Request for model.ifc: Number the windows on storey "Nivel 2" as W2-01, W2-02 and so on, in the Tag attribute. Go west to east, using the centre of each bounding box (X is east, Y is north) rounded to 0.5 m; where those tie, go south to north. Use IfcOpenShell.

First a look at what the model holds.

```python
import ifcopenshell
import ifcopenshell.util.element
import ifcopenshell.util.placement

model = ifcopenshell.open("model.ifc")
print(model.schema)
storey = next(s for s in model.by_type("IfcBuildingStorey") if s.Name == "Nivel 2")
windows = [e for e in ifcopenshell.util.element.get_decomposition(storey) if e.is_a("IfcWindow")]
for e in sorted(windows, key=lambda e: e.id()):
    origin = ifcopenshell.util.placement.get_local_placement(e.ObjectPlacement)[:3, 3]
    print(e.id(), e.Tag, e.Name, origin.round(2) + 0.0, sep=" | ")
```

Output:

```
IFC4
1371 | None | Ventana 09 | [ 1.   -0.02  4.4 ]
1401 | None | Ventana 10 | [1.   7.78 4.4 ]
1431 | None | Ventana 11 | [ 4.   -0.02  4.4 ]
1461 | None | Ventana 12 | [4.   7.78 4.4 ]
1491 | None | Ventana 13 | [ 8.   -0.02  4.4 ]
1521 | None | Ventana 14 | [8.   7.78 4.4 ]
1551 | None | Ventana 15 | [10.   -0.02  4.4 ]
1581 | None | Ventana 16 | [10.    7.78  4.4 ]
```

```python
import ifcopenshell
import ifcopenshell.geom
import ifcopenshell.util.element
import ifcopenshell.util.shape

model = ifcopenshell.open("model.ifc")
settings = ifcopenshell.geom.settings()
settings.set("use-world-coords", True)


def centre(element):
    shape = ifcopenshell.geom.create_shape(settings, element)
    return ifcopenshell.util.shape.get_bbox_centroid(shape.geometry)


storey = next(s for s in model.by_type("IfcBuildingStorey") if s.Name == "Nivel 2")
windows = [e for e in ifcopenshell.util.element.get_decomposition(storey) if e.is_a("IfcWindow")]

# Insertion points can sit at a corner or the storey origin, so sort by the geometry (in metres).
centres = {e: centre(e) for e in windows}
windows.sort(key=lambda e: (round(centres[e][0] / 0.5), centres[e][1]))

for i, e in enumerate(windows, start=1):
    number = f"W2-{i:02d}"
    e.Tag = number
    print(e.id(), number)

model.write("model_rev.ifc")
```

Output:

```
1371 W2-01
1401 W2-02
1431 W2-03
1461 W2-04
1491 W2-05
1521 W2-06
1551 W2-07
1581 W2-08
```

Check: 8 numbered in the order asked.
